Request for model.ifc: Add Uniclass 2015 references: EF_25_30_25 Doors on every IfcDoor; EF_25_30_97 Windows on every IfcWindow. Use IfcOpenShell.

First a look at what the model holds.

```python
import ifcopenshell

model = ifcopenshell.open("model.ifc")
print(model.schema)
print("classifications:", [c.Name for c in model.by_type("IfcClassification")])
for ifc_class in ("IfcDoor", "IfcRoof", "IfcStair", "IfcWall", "IfcWindow"):
    print(ifc_class, len(model.by_type(ifc_class)))
```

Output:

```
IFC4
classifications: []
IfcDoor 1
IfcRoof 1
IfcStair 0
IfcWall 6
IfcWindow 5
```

```python
import ifcopenshell
import ifcopenshell.api.classification

model = ifcopenshell.open("model.ifc")

system = ifcopenshell.api.classification.add_classification(model, classification="Uniclass 2015")

codes = {
    "IfcDoor": ("EF_25_30_25", "Doors"),
    "IfcWindow": ("EF_25_30_97", "Windows"),
}
for ifc_class, (code, name) in codes.items():
    products = model.by_type(ifc_class)
    ifcopenshell.api.classification.add_reference(
        model, products=products, classification=system, identification=code, name=name
    )
    print(code, len(products))

model.write("model_rev.ifc")
```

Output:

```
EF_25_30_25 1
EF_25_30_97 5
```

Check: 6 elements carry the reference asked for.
